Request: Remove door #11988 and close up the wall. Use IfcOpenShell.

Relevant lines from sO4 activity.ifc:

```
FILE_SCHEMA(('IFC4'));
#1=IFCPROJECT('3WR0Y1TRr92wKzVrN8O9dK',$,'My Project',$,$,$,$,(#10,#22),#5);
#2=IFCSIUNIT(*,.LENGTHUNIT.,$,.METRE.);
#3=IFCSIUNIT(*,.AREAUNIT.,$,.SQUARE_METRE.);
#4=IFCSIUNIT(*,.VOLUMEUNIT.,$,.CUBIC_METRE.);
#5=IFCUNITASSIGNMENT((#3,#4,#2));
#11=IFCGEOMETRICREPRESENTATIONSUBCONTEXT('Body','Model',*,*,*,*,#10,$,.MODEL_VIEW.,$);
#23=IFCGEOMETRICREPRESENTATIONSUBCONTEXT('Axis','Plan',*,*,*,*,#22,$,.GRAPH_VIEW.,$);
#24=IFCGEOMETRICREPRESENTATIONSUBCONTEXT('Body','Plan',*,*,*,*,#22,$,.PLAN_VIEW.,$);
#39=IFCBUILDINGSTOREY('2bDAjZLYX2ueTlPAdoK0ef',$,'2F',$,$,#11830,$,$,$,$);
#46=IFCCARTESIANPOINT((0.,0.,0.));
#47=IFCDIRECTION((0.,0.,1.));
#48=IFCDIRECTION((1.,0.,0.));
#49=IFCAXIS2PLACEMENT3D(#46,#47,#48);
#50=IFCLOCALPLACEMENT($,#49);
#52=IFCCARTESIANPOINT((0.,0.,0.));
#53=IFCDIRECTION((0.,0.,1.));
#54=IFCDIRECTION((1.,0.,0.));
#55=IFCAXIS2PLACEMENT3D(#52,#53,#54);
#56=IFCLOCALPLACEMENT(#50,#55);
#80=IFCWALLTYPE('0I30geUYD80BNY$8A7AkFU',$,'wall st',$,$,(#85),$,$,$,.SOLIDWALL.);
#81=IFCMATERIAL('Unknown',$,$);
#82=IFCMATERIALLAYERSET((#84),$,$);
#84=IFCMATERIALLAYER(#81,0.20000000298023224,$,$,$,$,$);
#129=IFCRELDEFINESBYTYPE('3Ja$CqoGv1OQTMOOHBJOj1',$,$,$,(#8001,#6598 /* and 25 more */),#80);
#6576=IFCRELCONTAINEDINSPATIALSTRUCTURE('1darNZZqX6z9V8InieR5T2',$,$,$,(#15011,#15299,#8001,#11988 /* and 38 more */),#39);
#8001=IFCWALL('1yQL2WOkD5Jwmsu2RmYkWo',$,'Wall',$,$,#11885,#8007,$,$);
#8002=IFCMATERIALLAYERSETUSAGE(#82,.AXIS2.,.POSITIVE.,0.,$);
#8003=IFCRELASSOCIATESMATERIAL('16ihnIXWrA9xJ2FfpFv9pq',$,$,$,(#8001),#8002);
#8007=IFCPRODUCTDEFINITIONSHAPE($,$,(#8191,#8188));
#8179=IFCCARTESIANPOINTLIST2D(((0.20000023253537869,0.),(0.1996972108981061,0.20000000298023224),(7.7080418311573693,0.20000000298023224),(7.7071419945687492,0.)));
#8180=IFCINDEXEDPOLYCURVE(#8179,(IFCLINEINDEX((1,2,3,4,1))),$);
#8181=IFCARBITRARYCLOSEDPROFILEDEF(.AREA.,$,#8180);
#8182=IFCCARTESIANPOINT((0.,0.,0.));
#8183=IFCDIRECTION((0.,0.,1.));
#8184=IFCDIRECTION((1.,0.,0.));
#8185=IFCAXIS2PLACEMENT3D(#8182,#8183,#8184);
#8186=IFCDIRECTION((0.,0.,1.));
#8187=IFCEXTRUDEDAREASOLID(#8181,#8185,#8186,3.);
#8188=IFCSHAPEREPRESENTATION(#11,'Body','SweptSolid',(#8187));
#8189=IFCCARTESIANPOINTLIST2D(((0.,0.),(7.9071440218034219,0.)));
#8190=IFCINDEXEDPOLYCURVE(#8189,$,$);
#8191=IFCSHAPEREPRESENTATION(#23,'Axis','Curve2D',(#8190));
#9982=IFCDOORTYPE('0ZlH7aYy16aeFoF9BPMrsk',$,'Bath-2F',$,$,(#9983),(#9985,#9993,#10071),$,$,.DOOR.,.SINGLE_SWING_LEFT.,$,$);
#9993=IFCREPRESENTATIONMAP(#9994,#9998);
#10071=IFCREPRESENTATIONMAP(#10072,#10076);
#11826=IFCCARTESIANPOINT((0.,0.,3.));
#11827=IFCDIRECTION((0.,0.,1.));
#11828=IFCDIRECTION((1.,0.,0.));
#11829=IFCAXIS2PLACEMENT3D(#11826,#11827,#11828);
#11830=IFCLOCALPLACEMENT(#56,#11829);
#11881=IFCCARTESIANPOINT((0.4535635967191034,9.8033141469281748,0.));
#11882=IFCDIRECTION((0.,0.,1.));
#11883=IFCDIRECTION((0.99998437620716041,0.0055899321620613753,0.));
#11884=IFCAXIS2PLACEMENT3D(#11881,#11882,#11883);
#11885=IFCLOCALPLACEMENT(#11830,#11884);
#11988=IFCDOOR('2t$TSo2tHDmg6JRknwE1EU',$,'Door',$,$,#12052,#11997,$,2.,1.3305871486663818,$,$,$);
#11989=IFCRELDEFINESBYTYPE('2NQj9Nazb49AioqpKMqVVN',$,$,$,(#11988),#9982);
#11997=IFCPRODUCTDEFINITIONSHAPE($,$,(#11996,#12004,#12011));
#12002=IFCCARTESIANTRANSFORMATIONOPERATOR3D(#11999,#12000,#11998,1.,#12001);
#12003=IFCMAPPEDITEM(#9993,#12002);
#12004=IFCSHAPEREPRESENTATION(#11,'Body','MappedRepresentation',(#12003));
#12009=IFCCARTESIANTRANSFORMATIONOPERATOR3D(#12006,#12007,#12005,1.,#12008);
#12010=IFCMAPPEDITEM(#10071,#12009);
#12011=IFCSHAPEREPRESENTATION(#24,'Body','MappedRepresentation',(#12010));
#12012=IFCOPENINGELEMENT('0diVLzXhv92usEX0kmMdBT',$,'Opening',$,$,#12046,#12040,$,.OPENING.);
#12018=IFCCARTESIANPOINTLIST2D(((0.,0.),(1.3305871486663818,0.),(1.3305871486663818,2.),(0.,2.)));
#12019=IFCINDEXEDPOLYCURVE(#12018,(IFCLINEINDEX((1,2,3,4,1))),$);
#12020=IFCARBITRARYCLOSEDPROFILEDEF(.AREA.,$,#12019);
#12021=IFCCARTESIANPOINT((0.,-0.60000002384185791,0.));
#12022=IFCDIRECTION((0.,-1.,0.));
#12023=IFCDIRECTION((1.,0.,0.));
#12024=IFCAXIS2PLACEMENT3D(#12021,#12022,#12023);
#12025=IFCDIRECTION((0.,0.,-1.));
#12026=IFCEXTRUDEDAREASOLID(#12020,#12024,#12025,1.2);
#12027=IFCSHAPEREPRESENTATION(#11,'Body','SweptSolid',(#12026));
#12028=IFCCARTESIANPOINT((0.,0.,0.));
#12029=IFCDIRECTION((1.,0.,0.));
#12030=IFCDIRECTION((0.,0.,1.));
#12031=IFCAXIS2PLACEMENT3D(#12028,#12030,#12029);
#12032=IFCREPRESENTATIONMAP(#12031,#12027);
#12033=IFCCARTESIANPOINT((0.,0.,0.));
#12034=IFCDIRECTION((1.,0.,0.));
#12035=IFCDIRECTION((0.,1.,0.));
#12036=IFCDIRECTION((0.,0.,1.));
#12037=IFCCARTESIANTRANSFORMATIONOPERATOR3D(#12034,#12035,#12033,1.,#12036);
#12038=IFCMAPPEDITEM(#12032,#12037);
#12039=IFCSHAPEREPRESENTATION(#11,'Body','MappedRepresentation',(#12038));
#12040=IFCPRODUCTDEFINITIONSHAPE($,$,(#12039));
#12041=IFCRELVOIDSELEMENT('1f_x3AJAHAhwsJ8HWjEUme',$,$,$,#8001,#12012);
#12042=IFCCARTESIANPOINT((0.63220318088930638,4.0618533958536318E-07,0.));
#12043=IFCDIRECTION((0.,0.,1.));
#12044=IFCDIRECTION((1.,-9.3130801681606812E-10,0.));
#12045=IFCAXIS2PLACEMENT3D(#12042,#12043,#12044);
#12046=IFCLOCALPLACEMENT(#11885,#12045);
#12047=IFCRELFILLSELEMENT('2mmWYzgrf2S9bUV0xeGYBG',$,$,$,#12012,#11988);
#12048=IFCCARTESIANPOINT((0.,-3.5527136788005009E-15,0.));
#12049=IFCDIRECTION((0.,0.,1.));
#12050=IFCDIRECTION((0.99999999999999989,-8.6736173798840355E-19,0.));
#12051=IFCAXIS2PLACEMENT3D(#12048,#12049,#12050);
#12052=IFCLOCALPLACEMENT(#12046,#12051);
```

```python
import ifcopenshell
import ifcopenshell.api.feature
import ifcopenshell.api.root
import ifcopenshell.geom
import ifcopenshell.util.shape

model = ifcopenshell.open("sO4 activity.ifc")
settings = ifcopenshell.geom.settings()


def volume(element):
    """Net volume in cubic metres, openings subtracted."""
    shape = ifcopenshell.geom.create_shape(settings, element)
    return ifcopenshell.util.shape.get_volume(shape.geometry)


door = model.by_id(11988)
opening = door.FillsVoids[0].RelatingOpeningElement
wall = opening.VoidsElements[0].RelatingBuildingElement
before = volume(wall)

ifcopenshell.api.root.remove_product(model, product=door)
ifcopenshell.api.feature.remove_feature(model, feature=opening)

after = volume(wall)

print(f"wall volume {before:.3f} -> {after:.3f} m3")

model.write("sO4 activity_updated.ifc")
```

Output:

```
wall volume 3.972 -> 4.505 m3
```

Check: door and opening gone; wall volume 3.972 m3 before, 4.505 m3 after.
